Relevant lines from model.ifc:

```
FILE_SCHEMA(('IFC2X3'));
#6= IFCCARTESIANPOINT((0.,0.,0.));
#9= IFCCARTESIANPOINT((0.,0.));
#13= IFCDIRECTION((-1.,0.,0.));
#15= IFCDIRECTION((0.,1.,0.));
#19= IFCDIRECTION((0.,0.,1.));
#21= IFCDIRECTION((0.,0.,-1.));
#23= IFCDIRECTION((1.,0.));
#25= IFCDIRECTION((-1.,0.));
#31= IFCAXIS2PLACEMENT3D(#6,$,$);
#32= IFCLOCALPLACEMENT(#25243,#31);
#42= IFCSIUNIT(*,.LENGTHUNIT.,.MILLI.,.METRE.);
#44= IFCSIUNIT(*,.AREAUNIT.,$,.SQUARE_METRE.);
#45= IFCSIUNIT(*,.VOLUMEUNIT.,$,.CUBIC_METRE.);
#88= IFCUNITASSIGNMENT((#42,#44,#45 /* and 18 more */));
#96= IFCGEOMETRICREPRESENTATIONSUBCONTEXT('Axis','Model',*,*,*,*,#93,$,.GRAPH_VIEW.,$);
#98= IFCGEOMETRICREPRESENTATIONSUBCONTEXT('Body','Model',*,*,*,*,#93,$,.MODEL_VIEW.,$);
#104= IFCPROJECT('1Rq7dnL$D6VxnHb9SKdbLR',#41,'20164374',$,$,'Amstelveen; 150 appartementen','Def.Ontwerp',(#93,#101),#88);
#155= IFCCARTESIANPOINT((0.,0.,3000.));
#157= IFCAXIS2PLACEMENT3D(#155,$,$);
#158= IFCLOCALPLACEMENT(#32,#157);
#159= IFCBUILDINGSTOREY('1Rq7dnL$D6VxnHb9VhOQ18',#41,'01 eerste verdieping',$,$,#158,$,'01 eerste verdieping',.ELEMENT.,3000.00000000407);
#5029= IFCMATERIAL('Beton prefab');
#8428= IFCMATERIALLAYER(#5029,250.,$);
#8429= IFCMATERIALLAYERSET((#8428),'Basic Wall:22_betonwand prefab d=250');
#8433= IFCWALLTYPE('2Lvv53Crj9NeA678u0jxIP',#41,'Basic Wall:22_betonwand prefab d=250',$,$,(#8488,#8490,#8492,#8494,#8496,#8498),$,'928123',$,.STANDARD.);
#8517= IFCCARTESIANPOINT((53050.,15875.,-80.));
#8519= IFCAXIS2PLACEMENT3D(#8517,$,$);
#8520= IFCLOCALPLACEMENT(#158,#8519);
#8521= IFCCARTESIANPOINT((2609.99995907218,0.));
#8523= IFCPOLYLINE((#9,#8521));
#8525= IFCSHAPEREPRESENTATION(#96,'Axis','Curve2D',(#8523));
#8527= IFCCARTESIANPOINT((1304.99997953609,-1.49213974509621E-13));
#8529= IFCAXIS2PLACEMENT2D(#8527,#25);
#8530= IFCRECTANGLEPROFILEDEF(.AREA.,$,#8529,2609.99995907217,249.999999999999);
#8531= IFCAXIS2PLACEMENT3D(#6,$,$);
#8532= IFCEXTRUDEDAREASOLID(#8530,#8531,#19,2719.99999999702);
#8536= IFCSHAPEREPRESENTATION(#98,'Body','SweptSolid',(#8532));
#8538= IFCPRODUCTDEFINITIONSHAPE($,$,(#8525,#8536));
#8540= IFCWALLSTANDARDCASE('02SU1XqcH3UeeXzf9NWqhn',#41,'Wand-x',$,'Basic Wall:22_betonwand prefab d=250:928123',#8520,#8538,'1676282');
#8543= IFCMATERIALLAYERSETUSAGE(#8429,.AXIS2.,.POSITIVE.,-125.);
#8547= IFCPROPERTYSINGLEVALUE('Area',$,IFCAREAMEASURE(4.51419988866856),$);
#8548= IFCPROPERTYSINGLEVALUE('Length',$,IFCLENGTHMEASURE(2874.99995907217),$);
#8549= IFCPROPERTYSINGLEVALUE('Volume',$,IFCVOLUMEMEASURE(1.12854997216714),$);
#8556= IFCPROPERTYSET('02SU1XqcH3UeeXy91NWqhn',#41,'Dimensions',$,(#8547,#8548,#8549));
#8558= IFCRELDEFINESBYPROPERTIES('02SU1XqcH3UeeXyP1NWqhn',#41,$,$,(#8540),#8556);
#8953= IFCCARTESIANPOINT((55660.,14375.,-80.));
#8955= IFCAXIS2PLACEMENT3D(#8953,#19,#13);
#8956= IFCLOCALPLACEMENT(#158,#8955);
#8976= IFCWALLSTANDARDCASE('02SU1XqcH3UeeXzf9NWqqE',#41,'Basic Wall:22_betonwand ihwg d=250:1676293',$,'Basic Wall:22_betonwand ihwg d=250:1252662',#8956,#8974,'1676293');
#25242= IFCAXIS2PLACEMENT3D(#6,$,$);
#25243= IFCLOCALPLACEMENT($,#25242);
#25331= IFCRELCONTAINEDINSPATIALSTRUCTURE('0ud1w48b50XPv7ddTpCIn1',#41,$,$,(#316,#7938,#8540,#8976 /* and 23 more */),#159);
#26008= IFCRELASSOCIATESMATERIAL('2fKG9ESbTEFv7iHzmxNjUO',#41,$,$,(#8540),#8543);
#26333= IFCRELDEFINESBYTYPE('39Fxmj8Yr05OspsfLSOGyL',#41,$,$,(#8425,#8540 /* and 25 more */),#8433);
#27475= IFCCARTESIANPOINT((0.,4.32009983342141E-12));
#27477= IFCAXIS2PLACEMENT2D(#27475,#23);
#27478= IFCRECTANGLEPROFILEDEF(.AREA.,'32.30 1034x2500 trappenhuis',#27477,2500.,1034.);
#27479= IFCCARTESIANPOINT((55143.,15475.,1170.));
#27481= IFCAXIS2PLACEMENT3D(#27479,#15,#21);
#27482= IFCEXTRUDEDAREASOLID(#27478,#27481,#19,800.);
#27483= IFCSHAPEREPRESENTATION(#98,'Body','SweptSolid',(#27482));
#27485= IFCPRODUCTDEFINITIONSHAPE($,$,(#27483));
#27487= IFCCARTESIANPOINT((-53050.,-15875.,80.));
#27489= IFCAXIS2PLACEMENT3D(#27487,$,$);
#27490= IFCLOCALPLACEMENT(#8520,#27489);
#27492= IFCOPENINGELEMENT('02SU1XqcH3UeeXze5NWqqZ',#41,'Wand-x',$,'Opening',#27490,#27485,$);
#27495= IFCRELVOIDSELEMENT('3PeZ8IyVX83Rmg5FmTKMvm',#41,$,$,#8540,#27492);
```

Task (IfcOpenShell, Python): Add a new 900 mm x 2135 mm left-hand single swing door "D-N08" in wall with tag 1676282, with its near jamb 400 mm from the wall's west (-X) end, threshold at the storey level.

```python
import numpy as np
import ifcopenshell
import ifcopenshell.api.feature
import ifcopenshell.api.geometry
import ifcopenshell.api.pset
import ifcopenshell.api.root
import ifcopenshell.api.spatial
import ifcopenshell.api.type
import ifcopenshell.geom
import ifcopenshell.util.element
import ifcopenshell.util.placement
import ifcopenshell.util.representation
import ifcopenshell.util.shape
import ifcopenshell.util.unit

model = ifcopenshell.open("model.ifc")
unit_scale = ifcopenshell.util.unit.calculate_unit_scale(model)
area_scale = ifcopenshell.util.unit.calculate_unit_scale(model, "AREAUNIT")
volume_scale = ifcopenshell.util.unit.calculate_unit_scale(model, "VOLUMEUNIT")
settings = ifcopenshell.geom.settings()


def volume(element):
    """Net volume in cubic metres, openings subtracted."""
    shape = ifcopenshell.geom.create_shape(settings, element)
    return ifcopenshell.util.shape.get_volume(shape.geometry)


wall = model.by_guid("02SU1XqcH3UeeXzf9NWqhn")
storey = ifcopenshell.util.element.get_container(wall, ifc_class="IfcBuildingStorey")
context = ifcopenshell.util.representation.get_context(model, "Model", "Body", "MODEL_VIEW")
before = volume(wall)

width, height, from_end, sill = 0.9, 2.135, 0.4, 0.0  # metres

# The wall runs along its own X axis, and the end named is its -X end.
wall_shape = ifcopenshell.geom.create_shape(settings, wall)
x, y, z = ifcopenshell.util.shape.get_vertices(wall_shape.geometry).T
start = x.min() + from_end
face, thickness = float(y.min()), float(y.max() - y.min())
wall_matrix = ifcopenshell.util.placement.get_local_placement(wall.ObjectPlacement)
level = ifcopenshell.util.placement.get_local_placement(storey.ObjectPlacement)[2, 3]


def in_wall(x, y):
    """Placement at x, y metres in the wall's axes, at sill height."""
    matrix = wall_matrix.copy()
    matrix[:, 3] = wall_matrix @ np.array([x / unit_scale, y / unit_scale, 0.0, 1.0])
    matrix[2, 3] = level + sill / unit_scale
    return matrix


# Opening: a box that overshoots both wall faces by 50 mm.
opening = ifcopenshell.api.root.create_entity(model, ifc_class="IfcOpeningElement")
box = ifcopenshell.api.geometry.add_wall_representation(
    model, context=context, length=width, height=height, thickness=thickness + 0.1
)
ifcopenshell.api.geometry.assign_representation(model, product=opening, representation=box)
ifcopenshell.api.geometry.edit_object_placement(model, product=opening, matrix=in_wall(start, face - 0.05), is_si=False)
ifcopenshell.api.feature.add_feature(model, feature=opening, element=wall)

door = ifcopenshell.api.root.create_entity(model, ifc_class="IfcDoor", name="D-N08")
door.OverallWidth, door.OverallHeight = width / unit_scale, height / unit_scale
body = ifcopenshell.api.geometry.add_door_representation(
    model,
    context=context,
    overall_width=door.OverallWidth,
    overall_height=door.OverallHeight,
    operation_type="SINGLE_SWING_LEFT",
    lining_properties={"LiningDepth": thickness / unit_scale, "ThresholdDepth": thickness / unit_scale},
)
ifcopenshell.api.geometry.assign_representation(model, product=door, representation=body)
ifcopenshell.api.spatial.assign_container(model, products=[door], relating_structure=storey)
fills = ifcopenshell.api.feature.add_filling(model, opening=opening, element=door)
fills.OwnerHistory = door.OwnerHistory  # required in IFC2X3

# IFC2X3 keeps the operation on the door style.
style = ifcopenshell.api.root.create_entity(model, ifc_class="IfcDoorStyle", name="D-N08")
style.OperationType, style.ConstructionType = "SINGLE_SWING_LEFT", "NOTDEFINED"
style.ParameterTakesPrecedence = style.Sizeable = False
ifcopenshell.api.type.assign_type(model, related_objects=[door], relating_type=style)

# The lining spans the wall, so the door starts at the wall face.
ifcopenshell.api.geometry.edit_object_placement(model, product=door, matrix=in_wall(start, face), is_si=False)

after = volume(wall)

# Update the wall's stored quantities.
pset = model.by_id(ifcopenshell.util.element.get_pset(wall, "Dimensions", should_inherit=False)["id"])
ifcopenshell.api.pset.edit_pset(model, pset=pset, properties={
    "Area": model.create_entity("IfcAreaMeasure", after / thickness / area_scale),
    "Volume": model.create_entity("IfcVolumeMeasure", after / volume_scale),
})

print(f"wall volume {before:.3f} -> {after:.3f} m3")

model.write("model_v2.ifc")
```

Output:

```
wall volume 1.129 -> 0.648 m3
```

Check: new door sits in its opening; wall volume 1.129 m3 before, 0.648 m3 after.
